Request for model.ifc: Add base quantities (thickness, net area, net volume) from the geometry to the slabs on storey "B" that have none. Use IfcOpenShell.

First a look at what the model holds.

```python
import ifcopenshell
import ifcopenshell.util.element
import ifcopenshell.util.unit

model = ifcopenshell.open("model.ifc")
print(model.schema)
for unit_type in ("LENGTHUNIT", "AREAUNIT", "VOLUMEUNIT"):
    print(unit_type, ifcopenshell.util.unit.calculate_unit_scale(model, unit_type))
storey = next(s for s in model.by_type("IfcBuildingStorey") if s.Name == "B")
slabs = [e for e in ifcopenshell.util.element.get_decomposition(storey) if e.is_a("IfcSlab")]
for e in sorted(slabs, key=lambda e: e.id()):
    print(e.id(), e.is_a(), e.Name, list(ifcopenshell.util.element.get_psets(e, qtos_only=True)), sep=" | ")
```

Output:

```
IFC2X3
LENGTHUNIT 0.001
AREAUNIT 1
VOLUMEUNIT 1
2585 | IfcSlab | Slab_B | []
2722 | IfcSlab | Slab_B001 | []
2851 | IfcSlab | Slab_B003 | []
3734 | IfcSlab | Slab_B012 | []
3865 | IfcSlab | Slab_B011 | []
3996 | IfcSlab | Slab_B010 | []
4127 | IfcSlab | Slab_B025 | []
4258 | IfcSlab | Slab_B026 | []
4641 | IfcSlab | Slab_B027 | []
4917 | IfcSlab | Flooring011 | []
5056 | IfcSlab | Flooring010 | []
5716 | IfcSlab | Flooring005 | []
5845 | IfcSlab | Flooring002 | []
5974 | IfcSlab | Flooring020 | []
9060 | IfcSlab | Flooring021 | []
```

```python
import ifcopenshell
import ifcopenshell.api.pset
import ifcopenshell.geom
import ifcopenshell.util.element
import ifcopenshell.util.shape
import ifcopenshell.util.unit

model = ifcopenshell.open("model.ifc")
unit_scale = ifcopenshell.util.unit.calculate_unit_scale(model)
area_scale = ifcopenshell.util.unit.calculate_unit_scale(model, "AREAUNIT")
volume_scale = ifcopenshell.util.unit.calculate_unit_scale(model, "VOLUMEUNIT")
settings = ifcopenshell.geom.settings()

storey = next(s for s in model.by_type("IfcBuildingStorey") if s.Name == "B")
slabs = [e for e in ifcopenshell.util.element.get_decomposition(storey) if e.is_a("IfcSlab")]

for e in sorted(slabs, key=lambda e: e.id()):
    if ifcopenshell.util.element.get_psets(e, qtos_only=True, should_inherit=False):
        continue
    # Geometry comes back in metres, in the element's own axes.
    shape = ifcopenshell.geom.create_shape(settings, e)
    values = {
        "Width": ifcopenshell.util.shape.get_z(shape.geometry) / unit_scale,
        "NetArea": ifcopenshell.util.shape.get_footprint_area(shape.geometry) / area_scale,
        "NetVolume": ifcopenshell.util.shape.get_volume(shape.geometry) / volume_scale,
    }
    qto = ifcopenshell.api.pset.add_qto(model, product=e, name="BaseQuantities")
    ifcopenshell.api.pset.edit_qto(model, qto=qto, properties=values)
    print(e.id(), {k: round(v, 3) for k, v in values.items()})

model.write("model-out.ifc")
```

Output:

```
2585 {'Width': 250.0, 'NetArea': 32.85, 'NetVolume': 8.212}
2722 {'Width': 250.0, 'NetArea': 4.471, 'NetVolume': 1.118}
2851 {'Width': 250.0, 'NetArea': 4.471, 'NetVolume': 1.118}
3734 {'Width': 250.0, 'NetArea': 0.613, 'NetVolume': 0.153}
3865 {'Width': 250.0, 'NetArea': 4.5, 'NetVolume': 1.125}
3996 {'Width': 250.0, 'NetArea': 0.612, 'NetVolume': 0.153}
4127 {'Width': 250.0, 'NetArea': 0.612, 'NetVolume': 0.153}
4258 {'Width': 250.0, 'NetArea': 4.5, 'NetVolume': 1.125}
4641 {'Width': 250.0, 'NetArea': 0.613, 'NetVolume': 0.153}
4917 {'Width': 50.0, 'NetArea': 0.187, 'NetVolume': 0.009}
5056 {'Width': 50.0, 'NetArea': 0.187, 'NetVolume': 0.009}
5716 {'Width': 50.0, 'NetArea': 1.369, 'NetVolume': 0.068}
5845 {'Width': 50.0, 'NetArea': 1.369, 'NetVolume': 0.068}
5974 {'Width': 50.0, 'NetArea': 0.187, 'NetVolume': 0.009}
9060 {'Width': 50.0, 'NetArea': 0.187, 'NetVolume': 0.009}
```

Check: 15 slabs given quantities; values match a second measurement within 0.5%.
